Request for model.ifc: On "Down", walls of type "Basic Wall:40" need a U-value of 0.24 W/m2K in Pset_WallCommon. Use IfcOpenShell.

First a look at what the model holds.

```python
import ifcopenshell
import ifcopenshell.util.element

model = ifcopenshell.open("model.ifc")
print(model.schema)
storey = next(s for s in model.by_type("IfcBuildingStorey") if s.Name == "Down")
walls = [e for e in ifcopenshell.util.element.get_decomposition(storey) if e.is_a("IfcWall")]
seen = {}
for e in walls:
    element_type = ifcopenshell.util.element.get_type(e)
    key = (element_type.Name if element_type != e and element_type else None, ifcopenshell.util.element.get_pset(e, "Pset_WallCommon", "ThermalTransmittance"))
    seen[key] = seen.get(key, 0) + 1
for (name, value), count in sorted(seen.items(), key=str):
    print(count, "x", name, "|", value)
```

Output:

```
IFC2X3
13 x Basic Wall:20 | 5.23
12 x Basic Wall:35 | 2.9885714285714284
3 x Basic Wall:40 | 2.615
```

```python
import ifcopenshell
import ifcopenshell.api.pset
import ifcopenshell.util.element

model = ifcopenshell.open("model.ifc")

storey = next(s for s in model.by_type("IfcBuildingStorey") if s.Name == "Down")
walls = [e for e in ifcopenshell.util.element.get_decomposition(storey) if e.is_a("IfcWall")]

count = 0
for e in walls:
    element_type = ifcopenshell.util.element.get_type(e)
    if element_type in (None, e) or element_type.Name != "Basic Wall:40":
        continue
    # add_pset returns the element's existing set when there is one.
    pset = ifcopenshell.api.pset.add_pset(model, product=e, name="Pset_WallCommon")
    ifcopenshell.api.pset.edit_pset(model, pset=pset, properties={"ThermalTransmittance": 0.24})
    count += 1

print(count, "walls updated")

model.write("model_updated.ifc")
```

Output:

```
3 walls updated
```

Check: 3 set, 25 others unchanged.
